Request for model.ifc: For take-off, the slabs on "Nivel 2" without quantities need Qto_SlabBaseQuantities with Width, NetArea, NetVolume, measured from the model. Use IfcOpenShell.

First a look at what the model holds.

```python
import ifcopenshell
import ifcopenshell.util.element
import ifcopenshell.util.unit

model = ifcopenshell.open("model.ifc")
print(model.schema)
for unit_type in ("LENGTHUNIT", "AREAUNIT", "VOLUMEUNIT"):
    print(unit_type, ifcopenshell.util.unit.calculate_unit_scale(model, unit_type))
storey = next(s for s in model.by_type("IfcBuildingStorey") if s.Name == "Nivel 2")
slabs = [e for e in ifcopenshell.util.element.get_decomposition(storey) if e.is_a("IfcSlab")]
for e in sorted(slabs, key=lambda e: e.id()):
    print(e.id(), e.is_a(), e.Name, list(ifcopenshell.util.element.get_psets(e, qtos_only=True)), sep=" | ")
```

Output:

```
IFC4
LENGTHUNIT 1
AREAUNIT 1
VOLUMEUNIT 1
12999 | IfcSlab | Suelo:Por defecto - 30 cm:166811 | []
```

```python
import ifcopenshell
import ifcopenshell.api.pset
import ifcopenshell.geom
import ifcopenshell.util.element
import ifcopenshell.util.shape
import ifcopenshell.util.unit

model = ifcopenshell.open("model.ifc")
unit_scale = ifcopenshell.util.unit.calculate_unit_scale(model)
area_scale = ifcopenshell.util.unit.calculate_unit_scale(model, "AREAUNIT")
volume_scale = ifcopenshell.util.unit.calculate_unit_scale(model, "VOLUMEUNIT")
settings = ifcopenshell.geom.settings()

storey = next(s for s in model.by_type("IfcBuildingStorey") if s.Name == "Nivel 2")
slabs = [e for e in ifcopenshell.util.element.get_decomposition(storey) if e.is_a("IfcSlab")]

for e in sorted(slabs, key=lambda e: e.id()):
    if ifcopenshell.util.element.get_psets(e, qtos_only=True, should_inherit=False):
        continue
    # Geometry comes back in metres, in the element's own axes.
    shape = ifcopenshell.geom.create_shape(settings, e)
    values = {
        "Width": ifcopenshell.util.shape.get_z(shape.geometry) / unit_scale,
        "NetArea": ifcopenshell.util.shape.get_footprint_area(shape.geometry) / area_scale,
        "NetVolume": ifcopenshell.util.shape.get_volume(shape.geometry) / volume_scale,
    }
    qto = ifcopenshell.api.pset.add_qto(model, product=e, name="Qto_SlabBaseQuantities")
    ifcopenshell.api.pset.edit_qto(model, qto=qto, properties=values)
    print(e.id(), {k: round(v, 3) for k, v in values.items()})

model.write("model-out.ifc")
```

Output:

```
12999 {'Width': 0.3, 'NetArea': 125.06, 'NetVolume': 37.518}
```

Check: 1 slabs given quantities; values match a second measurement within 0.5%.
